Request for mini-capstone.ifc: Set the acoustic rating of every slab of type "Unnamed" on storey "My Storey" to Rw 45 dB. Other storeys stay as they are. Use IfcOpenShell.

First a look at what the model holds.

```python
import ifcopenshell
import ifcopenshell.util.element

model = ifcopenshell.open("mini-capstone.ifc")
print(model.schema)
storey = next(s for s in model.by_type("IfcBuildingStorey") if s.Name == "My Storey")
slabs = [e for e in ifcopenshell.util.element.get_decomposition(storey) if e.is_a("IfcSlab")]
seen = {}
for e in slabs:
    element_type = ifcopenshell.util.element.get_type(e)
    key = (element_type.Name if element_type != e and element_type else None, ifcopenshell.util.element.get_pset(e, "Pset_SlabCommon", "AcousticRating"))
    seen[key] = seen.get(key, 0) + 1
for (name, value), count in sorted(seen.items(), key=str):
    print(count, "x", name, "|", value)
```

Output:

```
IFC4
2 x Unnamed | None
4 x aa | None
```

```python
import ifcopenshell
import ifcopenshell.api.pset
import ifcopenshell.util.element

model = ifcopenshell.open("mini-capstone.ifc")

storey = next(s for s in model.by_type("IfcBuildingStorey") if s.Name == "My Storey")
slabs = [e for e in ifcopenshell.util.element.get_decomposition(storey) if e.is_a("IfcSlab")]

count = 0
for e in slabs:
    element_type = ifcopenshell.util.element.get_type(e)
    if element_type in (None, e) or element_type.Name != "Unnamed":
        continue
    # add_pset returns the element's existing set when there is one.
    pset = ifcopenshell.api.pset.add_pset(model, product=e, name="Pset_SlabCommon")
    ifcopenshell.api.pset.edit_pset(model, pset=pset, properties={"AcousticRating": "Rw 45 dB"})
    count += 1

print(count, "slabs updated")

model.write("mini-capstone-out.ifc")
```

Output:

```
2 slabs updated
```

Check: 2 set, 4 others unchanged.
